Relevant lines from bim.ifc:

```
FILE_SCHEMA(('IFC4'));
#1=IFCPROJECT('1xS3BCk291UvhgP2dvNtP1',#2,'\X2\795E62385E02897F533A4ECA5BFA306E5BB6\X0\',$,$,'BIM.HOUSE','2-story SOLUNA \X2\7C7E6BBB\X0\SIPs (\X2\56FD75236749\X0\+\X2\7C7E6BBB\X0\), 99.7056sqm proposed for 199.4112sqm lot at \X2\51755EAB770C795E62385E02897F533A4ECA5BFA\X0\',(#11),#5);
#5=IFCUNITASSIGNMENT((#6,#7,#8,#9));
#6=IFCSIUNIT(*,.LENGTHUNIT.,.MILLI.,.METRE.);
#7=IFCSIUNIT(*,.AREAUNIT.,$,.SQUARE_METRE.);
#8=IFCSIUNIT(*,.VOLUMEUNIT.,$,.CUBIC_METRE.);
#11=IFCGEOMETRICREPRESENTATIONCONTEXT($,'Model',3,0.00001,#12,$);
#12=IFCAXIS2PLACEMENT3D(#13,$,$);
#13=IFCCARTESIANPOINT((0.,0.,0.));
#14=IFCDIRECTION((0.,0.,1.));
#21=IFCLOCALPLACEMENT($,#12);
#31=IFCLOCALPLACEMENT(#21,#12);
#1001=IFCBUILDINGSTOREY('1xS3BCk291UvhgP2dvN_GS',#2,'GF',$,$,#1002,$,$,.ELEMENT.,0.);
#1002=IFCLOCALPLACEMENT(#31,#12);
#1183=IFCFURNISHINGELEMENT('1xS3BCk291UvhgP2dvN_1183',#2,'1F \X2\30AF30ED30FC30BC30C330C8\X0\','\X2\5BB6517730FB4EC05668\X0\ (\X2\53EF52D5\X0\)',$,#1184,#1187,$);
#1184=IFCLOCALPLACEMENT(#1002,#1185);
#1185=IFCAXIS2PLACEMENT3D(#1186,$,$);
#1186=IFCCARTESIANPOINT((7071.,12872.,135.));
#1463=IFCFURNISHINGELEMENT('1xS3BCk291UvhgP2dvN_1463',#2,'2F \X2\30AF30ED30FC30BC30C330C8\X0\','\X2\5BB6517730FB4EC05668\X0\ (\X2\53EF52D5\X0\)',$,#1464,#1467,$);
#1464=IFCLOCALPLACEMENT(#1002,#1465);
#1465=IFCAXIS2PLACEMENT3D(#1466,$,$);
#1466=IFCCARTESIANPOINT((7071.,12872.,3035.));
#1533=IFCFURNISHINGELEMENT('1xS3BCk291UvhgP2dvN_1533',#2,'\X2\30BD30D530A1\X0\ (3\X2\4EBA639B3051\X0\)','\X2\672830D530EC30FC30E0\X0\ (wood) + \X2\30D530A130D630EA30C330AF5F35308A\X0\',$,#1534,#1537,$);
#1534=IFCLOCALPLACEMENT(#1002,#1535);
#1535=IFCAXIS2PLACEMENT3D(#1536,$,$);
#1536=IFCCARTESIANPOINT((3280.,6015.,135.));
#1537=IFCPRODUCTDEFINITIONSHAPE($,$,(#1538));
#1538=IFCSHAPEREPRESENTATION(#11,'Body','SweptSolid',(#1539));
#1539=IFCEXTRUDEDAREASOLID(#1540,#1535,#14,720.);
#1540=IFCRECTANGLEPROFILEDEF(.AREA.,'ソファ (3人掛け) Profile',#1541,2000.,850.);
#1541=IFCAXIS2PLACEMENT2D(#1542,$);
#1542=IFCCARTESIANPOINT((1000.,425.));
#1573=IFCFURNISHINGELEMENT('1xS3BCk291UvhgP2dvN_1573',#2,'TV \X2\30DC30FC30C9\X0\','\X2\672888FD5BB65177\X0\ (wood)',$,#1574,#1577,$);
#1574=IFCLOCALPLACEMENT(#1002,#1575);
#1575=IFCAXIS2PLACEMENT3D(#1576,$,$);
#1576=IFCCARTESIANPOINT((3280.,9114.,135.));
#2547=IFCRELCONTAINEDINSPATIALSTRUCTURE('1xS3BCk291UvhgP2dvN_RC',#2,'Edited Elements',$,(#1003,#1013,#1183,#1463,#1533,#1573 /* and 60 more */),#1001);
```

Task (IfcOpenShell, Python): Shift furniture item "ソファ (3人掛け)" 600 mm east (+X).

```python
import ifcopenshell
import ifcopenshell.api.geometry
import ifcopenshell.util.placement
import ifcopenshell.util.unit

model = ifcopenshell.open("bim.ifc")
unit_scale = ifcopenshell.util.unit.calculate_unit_scale(model)

item = model.by_guid("1xS3BCk291UvhgP2dvN_1533")
matrix = ifcopenshell.util.placement.get_local_placement(item.ObjectPlacement)
matrix[0, 3] += 0.6 / unit_scale
ifcopenshell.api.geometry.edit_object_placement(model, product=item, matrix=matrix, is_si=False)

print(ifcopenshell.util.placement.get_local_placement(item.ObjectPlacement).round(3) + 0.0)

model.write("bim_rev.ifc")
```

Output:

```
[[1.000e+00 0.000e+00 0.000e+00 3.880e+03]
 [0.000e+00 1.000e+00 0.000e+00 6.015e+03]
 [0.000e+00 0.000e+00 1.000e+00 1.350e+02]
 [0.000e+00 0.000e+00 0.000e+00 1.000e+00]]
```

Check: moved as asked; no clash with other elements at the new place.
